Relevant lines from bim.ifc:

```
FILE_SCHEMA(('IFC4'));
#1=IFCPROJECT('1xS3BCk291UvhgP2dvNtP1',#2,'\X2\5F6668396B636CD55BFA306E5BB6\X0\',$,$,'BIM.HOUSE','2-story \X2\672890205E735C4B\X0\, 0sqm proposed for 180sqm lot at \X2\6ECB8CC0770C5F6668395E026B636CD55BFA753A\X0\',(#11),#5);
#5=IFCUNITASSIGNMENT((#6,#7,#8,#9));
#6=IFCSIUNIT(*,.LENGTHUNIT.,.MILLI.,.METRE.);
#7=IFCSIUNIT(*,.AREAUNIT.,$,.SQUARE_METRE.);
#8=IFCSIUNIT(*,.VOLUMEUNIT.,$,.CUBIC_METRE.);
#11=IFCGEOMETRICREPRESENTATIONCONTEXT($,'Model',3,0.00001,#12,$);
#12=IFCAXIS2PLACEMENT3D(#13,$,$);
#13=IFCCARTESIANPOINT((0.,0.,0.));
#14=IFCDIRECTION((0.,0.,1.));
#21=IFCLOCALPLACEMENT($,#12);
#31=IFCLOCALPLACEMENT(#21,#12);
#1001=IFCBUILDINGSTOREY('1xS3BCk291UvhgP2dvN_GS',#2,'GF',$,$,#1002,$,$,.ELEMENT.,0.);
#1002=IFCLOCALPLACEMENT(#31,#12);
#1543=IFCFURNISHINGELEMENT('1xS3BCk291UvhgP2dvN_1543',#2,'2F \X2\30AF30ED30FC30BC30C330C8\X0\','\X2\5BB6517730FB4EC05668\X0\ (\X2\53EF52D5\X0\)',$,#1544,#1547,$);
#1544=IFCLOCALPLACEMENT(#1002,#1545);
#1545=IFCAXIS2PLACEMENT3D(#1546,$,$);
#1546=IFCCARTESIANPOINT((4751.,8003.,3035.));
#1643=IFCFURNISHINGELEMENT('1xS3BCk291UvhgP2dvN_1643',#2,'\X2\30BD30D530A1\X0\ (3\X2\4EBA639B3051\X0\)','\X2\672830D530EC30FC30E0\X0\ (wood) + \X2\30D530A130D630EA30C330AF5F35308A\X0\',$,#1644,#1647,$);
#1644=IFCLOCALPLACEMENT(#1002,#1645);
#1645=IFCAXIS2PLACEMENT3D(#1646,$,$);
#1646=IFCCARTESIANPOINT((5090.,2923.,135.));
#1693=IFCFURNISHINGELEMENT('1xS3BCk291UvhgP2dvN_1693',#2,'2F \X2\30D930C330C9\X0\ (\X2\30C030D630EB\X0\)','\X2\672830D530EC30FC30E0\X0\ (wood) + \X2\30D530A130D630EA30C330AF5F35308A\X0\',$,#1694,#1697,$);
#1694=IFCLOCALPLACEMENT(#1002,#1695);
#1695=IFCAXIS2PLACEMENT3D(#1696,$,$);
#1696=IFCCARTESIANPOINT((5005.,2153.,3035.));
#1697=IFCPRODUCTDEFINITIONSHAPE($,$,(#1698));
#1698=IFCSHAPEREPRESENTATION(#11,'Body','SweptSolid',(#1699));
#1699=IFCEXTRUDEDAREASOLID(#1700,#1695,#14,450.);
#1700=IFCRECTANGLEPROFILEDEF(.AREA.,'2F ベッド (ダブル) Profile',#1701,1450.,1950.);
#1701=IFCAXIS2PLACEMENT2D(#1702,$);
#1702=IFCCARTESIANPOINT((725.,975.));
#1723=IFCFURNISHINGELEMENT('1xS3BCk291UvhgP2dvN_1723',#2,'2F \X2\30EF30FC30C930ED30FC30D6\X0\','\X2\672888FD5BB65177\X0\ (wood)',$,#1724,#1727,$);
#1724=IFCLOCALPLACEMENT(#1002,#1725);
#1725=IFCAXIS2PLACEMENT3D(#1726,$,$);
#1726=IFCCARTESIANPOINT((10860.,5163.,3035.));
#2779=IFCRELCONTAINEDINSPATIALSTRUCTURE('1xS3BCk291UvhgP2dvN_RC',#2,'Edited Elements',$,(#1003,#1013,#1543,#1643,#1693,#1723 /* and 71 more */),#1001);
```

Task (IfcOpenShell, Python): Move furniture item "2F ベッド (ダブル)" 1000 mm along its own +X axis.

```python
import ifcopenshell
import ifcopenshell.api.geometry
import ifcopenshell.util.placement

model = ifcopenshell.open("bim.ifc")

item = model.by_guid("1xS3BCk291UvhgP2dvN_1693")
matrix = ifcopenshell.util.placement.get_local_placement(item.ObjectPlacement)
matrix[:3, 3] += matrix[:3, 0] * 1000.0
ifcopenshell.api.geometry.edit_object_placement(model, product=item, matrix=matrix, is_si=False)

print(ifcopenshell.util.placement.get_local_placement(item.ObjectPlacement).round(3) + 0.0)

model.write("bim_edited.ifc")
```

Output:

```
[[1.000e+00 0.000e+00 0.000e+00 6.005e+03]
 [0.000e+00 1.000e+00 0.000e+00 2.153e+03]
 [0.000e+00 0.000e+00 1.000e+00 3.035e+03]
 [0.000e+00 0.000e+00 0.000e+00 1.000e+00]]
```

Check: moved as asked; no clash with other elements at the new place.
